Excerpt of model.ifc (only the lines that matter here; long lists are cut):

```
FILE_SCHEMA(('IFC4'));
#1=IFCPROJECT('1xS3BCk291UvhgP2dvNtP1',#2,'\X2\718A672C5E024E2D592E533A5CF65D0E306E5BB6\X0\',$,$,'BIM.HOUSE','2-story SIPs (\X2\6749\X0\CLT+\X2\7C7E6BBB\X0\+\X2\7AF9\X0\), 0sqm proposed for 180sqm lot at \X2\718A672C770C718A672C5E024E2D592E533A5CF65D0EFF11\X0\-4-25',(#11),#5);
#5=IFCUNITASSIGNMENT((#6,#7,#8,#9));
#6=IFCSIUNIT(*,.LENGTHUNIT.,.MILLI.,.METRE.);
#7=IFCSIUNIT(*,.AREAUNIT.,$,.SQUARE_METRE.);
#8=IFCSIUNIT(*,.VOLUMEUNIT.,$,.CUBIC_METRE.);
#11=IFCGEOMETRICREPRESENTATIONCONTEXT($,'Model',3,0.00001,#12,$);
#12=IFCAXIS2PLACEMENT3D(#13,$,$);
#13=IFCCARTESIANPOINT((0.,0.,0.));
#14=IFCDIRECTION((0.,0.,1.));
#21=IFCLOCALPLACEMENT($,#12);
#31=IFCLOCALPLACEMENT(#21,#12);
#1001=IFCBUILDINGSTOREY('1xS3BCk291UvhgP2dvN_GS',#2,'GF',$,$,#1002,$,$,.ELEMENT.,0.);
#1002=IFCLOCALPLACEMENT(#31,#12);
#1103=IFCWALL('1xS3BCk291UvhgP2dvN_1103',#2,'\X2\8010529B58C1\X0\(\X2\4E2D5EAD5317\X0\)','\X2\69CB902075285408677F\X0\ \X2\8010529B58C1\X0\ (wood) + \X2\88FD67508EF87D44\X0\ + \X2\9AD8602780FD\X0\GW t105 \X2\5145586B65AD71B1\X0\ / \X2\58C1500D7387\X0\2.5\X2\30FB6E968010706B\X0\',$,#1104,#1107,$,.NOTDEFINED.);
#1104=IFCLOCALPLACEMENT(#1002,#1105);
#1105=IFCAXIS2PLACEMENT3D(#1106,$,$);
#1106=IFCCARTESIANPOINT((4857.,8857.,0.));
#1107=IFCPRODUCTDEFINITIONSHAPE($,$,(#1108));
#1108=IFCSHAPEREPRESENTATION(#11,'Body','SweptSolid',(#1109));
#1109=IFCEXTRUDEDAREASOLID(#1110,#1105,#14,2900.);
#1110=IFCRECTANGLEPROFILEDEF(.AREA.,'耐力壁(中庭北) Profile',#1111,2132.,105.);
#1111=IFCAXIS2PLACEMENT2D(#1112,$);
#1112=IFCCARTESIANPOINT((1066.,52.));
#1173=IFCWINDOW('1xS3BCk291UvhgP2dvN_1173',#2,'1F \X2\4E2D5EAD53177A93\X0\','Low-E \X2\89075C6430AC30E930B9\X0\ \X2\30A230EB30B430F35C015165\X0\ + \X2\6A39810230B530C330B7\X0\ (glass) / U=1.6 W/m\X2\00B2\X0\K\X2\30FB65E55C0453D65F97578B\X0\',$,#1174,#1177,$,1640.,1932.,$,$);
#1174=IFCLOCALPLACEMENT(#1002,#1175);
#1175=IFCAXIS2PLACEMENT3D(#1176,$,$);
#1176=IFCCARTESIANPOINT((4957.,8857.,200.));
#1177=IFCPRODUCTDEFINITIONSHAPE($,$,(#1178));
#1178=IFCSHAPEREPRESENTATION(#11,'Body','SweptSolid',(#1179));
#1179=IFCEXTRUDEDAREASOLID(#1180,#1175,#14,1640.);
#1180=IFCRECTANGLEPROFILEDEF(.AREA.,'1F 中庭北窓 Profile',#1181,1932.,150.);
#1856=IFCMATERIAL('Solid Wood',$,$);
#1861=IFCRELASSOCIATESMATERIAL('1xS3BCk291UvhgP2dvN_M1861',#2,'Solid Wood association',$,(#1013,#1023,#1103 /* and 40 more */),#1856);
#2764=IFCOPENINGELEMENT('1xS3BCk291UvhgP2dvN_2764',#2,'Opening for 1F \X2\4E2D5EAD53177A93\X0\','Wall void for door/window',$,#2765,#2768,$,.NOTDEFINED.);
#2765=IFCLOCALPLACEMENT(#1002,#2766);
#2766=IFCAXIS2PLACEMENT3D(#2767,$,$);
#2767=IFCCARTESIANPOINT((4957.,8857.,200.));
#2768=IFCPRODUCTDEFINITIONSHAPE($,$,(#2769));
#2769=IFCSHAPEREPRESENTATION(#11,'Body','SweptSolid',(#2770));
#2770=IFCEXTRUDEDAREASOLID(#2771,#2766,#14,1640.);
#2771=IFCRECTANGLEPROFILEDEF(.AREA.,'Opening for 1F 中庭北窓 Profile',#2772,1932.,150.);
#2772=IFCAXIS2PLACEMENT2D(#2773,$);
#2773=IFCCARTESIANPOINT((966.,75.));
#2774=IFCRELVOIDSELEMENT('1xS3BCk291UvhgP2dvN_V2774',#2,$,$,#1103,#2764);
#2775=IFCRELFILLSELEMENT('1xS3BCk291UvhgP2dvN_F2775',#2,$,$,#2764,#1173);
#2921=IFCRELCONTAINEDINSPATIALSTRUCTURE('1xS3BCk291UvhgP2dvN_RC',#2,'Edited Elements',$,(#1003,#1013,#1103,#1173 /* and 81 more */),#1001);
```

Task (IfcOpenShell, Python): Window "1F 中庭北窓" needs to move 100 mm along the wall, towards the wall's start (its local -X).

```python
import ifcopenshell
import ifcopenshell.api.geometry
import ifcopenshell.util.placement
import ifcopenshell.util.unit

model = ifcopenshell.open("model.ifc")
unit_scale = ifcopenshell.util.unit.calculate_unit_scale(model)

window = model.by_guid("1xS3BCk291UvhgP2dvN_1173")
opening = window.FillsVoids[0].RelatingOpeningElement
wall = opening.VoidsElements[0].RelatingBuildingElement

wall_matrix = ifcopenshell.util.placement.get_local_placement(wall.ObjectPlacement)
shift = wall_matrix[:3, 0] * -0.1 / unit_scale
before = ifcopenshell.util.placement.get_local_placement(window.ObjectPlacement)[:3, 3].copy()

# The window is not placed relative to its opening, so move both.
for product in (opening, window):
    matrix = ifcopenshell.util.placement.get_local_placement(product.ObjectPlacement)
    matrix[:3, 3] += shift
    ifcopenshell.api.geometry.edit_object_placement(model, product=product, matrix=matrix, is_si=False)

after = ifcopenshell.util.placement.get_local_placement(window.ObjectPlacement)[:3, 3]
print("window moved by", (after - before).round(3) + 0.0)

model.write("model_v2.ifc")
```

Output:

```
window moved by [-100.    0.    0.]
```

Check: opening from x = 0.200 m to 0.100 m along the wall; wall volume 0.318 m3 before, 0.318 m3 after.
